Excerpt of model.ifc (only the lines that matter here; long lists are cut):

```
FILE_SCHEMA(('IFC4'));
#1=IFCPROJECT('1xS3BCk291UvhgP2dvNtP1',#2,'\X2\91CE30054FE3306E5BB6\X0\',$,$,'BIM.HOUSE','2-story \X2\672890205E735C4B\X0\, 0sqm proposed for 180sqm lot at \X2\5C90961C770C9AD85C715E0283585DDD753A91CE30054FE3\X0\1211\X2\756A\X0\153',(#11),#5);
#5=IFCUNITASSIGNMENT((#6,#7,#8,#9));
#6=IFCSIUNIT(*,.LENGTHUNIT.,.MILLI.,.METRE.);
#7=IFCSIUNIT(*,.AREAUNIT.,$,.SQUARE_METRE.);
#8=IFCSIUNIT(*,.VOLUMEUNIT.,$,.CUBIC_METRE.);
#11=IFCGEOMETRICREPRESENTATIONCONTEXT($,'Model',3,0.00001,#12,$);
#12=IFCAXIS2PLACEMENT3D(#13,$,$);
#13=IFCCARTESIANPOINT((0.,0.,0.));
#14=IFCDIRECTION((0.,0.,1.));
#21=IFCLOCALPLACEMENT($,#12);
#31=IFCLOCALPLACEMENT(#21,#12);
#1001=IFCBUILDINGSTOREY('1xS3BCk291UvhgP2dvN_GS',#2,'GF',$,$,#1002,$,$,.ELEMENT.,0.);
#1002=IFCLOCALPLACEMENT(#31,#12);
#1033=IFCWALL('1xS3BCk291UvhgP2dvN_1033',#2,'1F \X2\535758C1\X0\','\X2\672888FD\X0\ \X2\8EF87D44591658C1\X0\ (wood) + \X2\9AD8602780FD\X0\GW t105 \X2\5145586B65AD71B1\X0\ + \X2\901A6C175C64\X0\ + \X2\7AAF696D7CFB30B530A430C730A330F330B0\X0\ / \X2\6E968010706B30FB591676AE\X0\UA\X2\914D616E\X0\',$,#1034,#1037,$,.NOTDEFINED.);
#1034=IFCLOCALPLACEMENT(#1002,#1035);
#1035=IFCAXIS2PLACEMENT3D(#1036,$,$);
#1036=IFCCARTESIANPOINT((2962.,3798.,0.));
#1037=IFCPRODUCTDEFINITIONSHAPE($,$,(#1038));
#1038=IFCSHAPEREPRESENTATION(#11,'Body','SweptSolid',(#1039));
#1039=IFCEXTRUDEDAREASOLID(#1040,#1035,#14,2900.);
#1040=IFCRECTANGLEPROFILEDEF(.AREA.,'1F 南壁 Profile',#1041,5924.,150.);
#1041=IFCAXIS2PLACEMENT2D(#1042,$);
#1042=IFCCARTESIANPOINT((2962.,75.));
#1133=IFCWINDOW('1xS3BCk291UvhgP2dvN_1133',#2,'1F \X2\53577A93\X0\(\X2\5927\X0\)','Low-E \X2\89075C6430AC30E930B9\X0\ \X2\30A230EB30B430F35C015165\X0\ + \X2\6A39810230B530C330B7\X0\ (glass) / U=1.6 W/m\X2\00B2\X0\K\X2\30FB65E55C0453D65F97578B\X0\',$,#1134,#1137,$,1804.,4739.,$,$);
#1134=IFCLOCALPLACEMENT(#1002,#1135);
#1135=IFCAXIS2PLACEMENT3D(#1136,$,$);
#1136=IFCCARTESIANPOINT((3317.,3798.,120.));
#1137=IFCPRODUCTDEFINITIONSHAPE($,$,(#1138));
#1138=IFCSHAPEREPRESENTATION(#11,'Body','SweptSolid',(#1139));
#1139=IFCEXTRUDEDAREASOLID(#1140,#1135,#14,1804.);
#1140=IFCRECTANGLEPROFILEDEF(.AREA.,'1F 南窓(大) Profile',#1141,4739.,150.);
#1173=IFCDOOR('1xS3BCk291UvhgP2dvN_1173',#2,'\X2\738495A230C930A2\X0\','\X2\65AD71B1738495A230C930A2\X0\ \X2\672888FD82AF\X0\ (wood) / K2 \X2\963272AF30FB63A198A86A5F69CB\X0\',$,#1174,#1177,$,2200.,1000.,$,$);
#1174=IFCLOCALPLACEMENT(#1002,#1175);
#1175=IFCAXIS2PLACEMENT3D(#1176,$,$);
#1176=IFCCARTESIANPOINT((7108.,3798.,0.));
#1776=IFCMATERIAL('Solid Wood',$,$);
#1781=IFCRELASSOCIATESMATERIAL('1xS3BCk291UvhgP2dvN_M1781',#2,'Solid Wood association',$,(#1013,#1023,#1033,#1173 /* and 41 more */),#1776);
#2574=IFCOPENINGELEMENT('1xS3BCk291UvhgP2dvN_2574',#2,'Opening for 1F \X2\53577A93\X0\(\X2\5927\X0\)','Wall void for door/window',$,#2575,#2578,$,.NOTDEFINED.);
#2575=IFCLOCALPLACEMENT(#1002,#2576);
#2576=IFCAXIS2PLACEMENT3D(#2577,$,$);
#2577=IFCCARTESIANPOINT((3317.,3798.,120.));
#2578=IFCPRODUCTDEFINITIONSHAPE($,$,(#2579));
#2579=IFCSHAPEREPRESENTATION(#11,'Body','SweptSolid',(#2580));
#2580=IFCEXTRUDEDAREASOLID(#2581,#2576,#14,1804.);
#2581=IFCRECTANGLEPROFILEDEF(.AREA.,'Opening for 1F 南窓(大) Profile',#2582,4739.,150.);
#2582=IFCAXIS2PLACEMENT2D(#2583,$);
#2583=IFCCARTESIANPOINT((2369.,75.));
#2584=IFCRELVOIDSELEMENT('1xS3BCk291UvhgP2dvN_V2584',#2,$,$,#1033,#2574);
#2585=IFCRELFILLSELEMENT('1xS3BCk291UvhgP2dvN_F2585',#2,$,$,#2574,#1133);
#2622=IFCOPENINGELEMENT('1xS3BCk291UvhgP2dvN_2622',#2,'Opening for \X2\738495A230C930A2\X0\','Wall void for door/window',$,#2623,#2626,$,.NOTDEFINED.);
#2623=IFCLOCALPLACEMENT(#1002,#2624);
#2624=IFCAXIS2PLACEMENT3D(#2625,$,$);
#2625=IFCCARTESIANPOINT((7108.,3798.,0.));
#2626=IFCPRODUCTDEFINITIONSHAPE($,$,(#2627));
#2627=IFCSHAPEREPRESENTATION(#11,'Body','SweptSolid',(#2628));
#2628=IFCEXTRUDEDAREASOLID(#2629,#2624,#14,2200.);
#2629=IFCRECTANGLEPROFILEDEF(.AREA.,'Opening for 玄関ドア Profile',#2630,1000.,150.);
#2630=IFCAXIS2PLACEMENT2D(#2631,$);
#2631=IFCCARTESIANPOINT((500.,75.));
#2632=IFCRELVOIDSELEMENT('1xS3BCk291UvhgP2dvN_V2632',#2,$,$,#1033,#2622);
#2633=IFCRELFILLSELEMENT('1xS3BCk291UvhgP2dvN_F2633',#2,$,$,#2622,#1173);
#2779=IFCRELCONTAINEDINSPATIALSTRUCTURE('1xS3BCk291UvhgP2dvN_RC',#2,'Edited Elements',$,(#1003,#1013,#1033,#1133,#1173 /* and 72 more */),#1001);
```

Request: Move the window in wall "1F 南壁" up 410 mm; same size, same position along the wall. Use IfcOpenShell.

```python
import numpy as np
import ifcopenshell
import ifcopenshell.api.geometry
import ifcopenshell.util.placement
import ifcopenshell.util.unit

model = ifcopenshell.open("model.ifc")
unit_scale = ifcopenshell.util.unit.calculate_unit_scale(model)

window = model.by_guid("1xS3BCk291UvhgP2dvN_1133")
opening = window.FillsVoids[0].RelatingOpeningElement
dz = 0.41 / unit_scale

shift = np.array([0.0, 0.0, dz])
# The window is not placed relative to its opening, so move both.
for product in (opening, window):
    matrix = ifcopenshell.util.placement.get_local_placement(product.ObjectPlacement)
    matrix[:3, 3] += shift
    ifcopenshell.api.geometry.edit_object_placement(model, product=product, matrix=matrix, is_si=False)

print(f"moved by {dz * unit_scale:+.3f} m")

model.write("model_edited.ifc")
```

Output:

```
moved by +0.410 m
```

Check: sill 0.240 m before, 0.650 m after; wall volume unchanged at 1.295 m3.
